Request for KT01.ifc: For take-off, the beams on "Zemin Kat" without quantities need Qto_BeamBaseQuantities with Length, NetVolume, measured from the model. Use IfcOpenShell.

First a look at what the model holds.

```python
import ifcopenshell
import ifcopenshell.util.element
import ifcopenshell.util.unit

model = ifcopenshell.open("KT01.ifc")
print(model.schema)
for unit_type in ("LENGTHUNIT", "AREAUNIT", "VOLUMEUNIT"):
    print(unit_type, ifcopenshell.util.unit.calculate_unit_scale(model, unit_type))
storey = next(s for s in model.by_type("IfcBuildingStorey") if s.Name == "Zemin Kat")
beams = [e for e in ifcopenshell.util.element.get_decomposition(storey) if e.is_a("IfcBeam")]
for e in sorted(beams, key=lambda e: e.id()):
    print(e.id(), e.is_a(), e.Name, list(ifcopenshell.util.element.get_psets(e, qtos_only=True)), sep=" | ")
```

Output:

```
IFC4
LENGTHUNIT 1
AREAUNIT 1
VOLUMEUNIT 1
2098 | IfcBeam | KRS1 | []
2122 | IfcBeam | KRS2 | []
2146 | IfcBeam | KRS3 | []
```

```python
import ifcopenshell
import ifcopenshell.api.pset
import ifcopenshell.geom
import ifcopenshell.util.element
import ifcopenshell.util.shape
import ifcopenshell.util.unit

model = ifcopenshell.open("KT01.ifc")
unit_scale = ifcopenshell.util.unit.calculate_unit_scale(model)
volume_scale = ifcopenshell.util.unit.calculate_unit_scale(model, "VOLUMEUNIT")
settings = ifcopenshell.geom.settings()

storey = next(s for s in model.by_type("IfcBuildingStorey") if s.Name == "Zemin Kat")
beams = [e for e in ifcopenshell.util.element.get_decomposition(storey) if e.is_a("IfcBeam")]

for e in sorted(beams, key=lambda e: e.id()):
    if ifcopenshell.util.element.get_psets(e, qtos_only=True, should_inherit=False):
        continue
    # Geometry comes back in metres, in the element's own axes.
    shape = ifcopenshell.geom.create_shape(settings, e)
    values = {
        "Length": ifcopenshell.util.shape.get_max_xyz(shape.geometry) / unit_scale,
        "NetVolume": ifcopenshell.util.shape.get_volume(shape.geometry) / volume_scale,
    }
    qto = ifcopenshell.api.pset.add_qto(model, product=e, name="Qto_BeamBaseQuantities")
    ifcopenshell.api.pset.edit_qto(model, qto=qto, properties=values)
    print(e.id(), {k: round(v, 3) for k, v in values.items()})

model.write("KT01_v2.ifc")
```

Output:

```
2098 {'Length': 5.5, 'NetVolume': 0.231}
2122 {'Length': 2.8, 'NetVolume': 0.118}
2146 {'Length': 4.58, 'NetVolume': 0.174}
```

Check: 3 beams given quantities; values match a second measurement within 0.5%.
